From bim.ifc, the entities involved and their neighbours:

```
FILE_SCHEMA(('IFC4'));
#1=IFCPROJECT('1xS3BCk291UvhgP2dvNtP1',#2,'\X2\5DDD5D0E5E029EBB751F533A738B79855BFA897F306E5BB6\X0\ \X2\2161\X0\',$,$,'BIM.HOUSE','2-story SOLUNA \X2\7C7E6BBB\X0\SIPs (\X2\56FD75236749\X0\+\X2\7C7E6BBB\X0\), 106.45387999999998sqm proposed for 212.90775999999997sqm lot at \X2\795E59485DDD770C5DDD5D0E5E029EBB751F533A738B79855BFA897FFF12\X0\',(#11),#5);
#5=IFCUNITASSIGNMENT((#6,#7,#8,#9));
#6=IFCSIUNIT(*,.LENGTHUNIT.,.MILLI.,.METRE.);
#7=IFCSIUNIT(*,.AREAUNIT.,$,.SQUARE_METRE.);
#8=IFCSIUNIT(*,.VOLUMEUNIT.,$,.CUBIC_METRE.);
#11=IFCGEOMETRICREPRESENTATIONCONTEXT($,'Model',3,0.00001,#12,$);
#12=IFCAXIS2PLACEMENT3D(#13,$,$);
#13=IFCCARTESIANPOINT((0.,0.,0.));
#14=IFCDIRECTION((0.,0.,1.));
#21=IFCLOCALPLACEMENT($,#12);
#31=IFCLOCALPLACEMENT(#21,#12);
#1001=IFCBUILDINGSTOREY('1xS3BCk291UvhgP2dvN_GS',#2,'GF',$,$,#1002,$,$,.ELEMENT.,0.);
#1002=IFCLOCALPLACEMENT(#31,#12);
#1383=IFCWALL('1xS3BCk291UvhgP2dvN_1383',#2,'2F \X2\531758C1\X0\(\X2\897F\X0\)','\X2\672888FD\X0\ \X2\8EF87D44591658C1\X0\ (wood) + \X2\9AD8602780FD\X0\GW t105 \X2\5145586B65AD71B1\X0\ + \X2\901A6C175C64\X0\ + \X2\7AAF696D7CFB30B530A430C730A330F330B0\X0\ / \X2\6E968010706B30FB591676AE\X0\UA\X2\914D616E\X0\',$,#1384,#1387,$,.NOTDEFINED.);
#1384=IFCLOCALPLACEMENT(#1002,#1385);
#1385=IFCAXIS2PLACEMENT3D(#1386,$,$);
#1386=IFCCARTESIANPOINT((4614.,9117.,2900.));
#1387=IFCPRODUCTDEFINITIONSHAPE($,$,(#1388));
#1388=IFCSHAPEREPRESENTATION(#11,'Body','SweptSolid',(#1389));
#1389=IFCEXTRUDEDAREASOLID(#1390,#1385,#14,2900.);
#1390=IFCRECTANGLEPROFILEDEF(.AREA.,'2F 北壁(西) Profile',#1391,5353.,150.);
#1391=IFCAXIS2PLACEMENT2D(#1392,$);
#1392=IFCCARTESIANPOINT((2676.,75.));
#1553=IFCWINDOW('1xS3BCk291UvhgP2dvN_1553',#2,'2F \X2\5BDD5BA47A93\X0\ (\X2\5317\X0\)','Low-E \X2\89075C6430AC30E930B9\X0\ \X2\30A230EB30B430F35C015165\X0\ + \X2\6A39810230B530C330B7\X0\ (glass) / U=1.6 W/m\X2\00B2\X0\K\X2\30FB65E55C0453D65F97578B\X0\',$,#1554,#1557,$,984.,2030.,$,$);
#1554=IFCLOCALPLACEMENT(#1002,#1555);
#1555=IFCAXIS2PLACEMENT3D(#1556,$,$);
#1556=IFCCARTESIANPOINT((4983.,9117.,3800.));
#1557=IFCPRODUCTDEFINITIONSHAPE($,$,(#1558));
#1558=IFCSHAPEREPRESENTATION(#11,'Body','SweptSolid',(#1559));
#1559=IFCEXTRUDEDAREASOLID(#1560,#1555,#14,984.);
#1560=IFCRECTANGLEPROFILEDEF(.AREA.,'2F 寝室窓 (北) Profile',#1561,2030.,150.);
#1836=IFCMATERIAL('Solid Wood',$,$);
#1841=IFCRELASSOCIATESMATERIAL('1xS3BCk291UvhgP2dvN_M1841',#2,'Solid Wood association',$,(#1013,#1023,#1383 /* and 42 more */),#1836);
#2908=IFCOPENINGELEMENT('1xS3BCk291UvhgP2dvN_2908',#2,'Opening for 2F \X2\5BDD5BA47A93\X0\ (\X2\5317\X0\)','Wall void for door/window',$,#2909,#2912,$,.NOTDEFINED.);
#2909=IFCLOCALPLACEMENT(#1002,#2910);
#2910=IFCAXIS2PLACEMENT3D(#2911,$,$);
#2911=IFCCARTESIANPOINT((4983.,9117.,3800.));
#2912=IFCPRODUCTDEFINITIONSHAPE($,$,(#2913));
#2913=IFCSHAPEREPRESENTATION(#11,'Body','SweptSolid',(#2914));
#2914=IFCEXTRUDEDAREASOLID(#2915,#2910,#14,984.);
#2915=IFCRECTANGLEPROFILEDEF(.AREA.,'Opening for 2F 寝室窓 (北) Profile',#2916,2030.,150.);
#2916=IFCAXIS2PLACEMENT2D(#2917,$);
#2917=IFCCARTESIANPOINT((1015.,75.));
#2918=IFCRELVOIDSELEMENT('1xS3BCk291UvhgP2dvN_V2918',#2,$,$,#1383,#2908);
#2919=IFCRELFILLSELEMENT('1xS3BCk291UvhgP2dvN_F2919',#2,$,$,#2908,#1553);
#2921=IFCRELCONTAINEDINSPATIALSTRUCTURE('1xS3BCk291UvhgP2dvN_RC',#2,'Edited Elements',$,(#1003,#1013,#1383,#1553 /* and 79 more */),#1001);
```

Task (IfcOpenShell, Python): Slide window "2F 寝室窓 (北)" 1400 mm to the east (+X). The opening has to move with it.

```python
import ifcopenshell
import ifcopenshell.api.geometry
import ifcopenshell.util.placement

model = ifcopenshell.open("bim.ifc")

window = model.by_guid("1xS3BCk291UvhgP2dvN_1553")
opening = window.FillsVoids[0].RelatingOpeningElement
wall = opening.VoidsElements[0].RelatingBuildingElement

wall_matrix = ifcopenshell.util.placement.get_local_placement(wall.ObjectPlacement)
shift = wall_matrix[:3, 0] * 1400.0
before = ifcopenshell.util.placement.get_local_placement(window.ObjectPlacement)[:3, 3].copy()

# The window is not placed relative to its opening, so move both.
for product in (opening, window):
    matrix = ifcopenshell.util.placement.get_local_placement(product.ObjectPlacement)
    matrix[:3, 3] += shift
    ifcopenshell.api.geometry.edit_object_placement(model, product=product, matrix=matrix, is_si=False)

after = ifcopenshell.util.placement.get_local_placement(window.ObjectPlacement)[:3, 3]
print("window moved by", (after - before).round(3) + 0.0)

model.write("bim-out.ifc")
```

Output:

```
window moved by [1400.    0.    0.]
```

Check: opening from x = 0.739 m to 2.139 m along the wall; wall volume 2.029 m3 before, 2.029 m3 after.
